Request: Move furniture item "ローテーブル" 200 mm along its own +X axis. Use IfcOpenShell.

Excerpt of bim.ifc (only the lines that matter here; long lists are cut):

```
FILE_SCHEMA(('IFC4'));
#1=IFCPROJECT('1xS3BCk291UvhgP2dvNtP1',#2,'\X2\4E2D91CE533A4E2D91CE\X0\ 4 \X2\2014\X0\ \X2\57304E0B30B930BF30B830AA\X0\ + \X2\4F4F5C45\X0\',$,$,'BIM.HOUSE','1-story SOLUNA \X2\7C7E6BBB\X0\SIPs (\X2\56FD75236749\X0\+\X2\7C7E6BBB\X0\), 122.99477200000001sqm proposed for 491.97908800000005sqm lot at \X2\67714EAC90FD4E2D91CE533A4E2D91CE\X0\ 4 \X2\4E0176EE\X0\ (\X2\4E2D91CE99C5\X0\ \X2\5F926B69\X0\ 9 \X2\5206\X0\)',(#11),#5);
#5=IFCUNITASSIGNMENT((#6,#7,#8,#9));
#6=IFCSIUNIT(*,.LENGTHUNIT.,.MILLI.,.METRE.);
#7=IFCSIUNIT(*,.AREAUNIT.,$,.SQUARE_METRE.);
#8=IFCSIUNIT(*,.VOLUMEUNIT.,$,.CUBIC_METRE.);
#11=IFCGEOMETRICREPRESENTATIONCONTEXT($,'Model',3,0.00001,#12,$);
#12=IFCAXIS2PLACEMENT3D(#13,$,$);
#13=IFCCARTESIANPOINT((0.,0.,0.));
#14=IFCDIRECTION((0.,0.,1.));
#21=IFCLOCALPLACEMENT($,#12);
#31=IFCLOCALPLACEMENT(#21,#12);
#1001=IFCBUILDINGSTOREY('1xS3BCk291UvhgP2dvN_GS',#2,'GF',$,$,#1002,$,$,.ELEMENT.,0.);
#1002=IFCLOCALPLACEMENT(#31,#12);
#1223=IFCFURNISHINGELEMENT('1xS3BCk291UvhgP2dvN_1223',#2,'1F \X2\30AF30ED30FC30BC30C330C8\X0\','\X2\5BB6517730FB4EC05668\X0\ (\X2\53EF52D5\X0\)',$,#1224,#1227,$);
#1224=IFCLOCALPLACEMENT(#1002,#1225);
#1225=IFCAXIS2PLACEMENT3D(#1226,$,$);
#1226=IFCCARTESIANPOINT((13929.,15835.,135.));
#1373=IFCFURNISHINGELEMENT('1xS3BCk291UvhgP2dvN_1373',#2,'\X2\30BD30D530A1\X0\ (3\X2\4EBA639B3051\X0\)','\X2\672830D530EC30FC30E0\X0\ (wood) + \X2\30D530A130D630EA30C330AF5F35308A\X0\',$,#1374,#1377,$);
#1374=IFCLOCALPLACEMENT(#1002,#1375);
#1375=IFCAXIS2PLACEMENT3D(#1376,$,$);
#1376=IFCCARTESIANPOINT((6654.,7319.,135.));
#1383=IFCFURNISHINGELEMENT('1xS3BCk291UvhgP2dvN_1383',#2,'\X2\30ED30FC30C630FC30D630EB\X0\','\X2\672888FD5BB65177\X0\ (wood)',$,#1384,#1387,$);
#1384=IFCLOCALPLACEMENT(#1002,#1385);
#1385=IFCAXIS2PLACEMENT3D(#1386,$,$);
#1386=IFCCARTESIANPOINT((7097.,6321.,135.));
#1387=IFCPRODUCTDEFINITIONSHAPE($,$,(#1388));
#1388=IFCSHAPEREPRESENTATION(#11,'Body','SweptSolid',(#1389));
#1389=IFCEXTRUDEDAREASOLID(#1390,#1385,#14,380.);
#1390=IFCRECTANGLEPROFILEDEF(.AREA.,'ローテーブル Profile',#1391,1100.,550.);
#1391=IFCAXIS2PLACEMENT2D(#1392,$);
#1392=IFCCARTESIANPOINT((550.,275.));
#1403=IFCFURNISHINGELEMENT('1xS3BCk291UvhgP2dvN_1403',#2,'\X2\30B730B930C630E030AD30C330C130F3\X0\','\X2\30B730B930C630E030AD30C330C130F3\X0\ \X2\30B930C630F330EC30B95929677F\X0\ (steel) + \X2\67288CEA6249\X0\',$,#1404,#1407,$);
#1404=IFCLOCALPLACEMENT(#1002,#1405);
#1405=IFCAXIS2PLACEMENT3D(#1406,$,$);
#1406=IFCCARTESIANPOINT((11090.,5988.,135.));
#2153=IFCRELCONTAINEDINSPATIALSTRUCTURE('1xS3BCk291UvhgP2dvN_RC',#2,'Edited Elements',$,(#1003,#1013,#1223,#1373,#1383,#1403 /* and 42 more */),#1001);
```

```python
import ifcopenshell
import ifcopenshell.api.geometry
import ifcopenshell.util.placement
import ifcopenshell.util.unit

model = ifcopenshell.open("bim.ifc")
unit_scale = ifcopenshell.util.unit.calculate_unit_scale(model)

item = model.by_id(1383)
matrix = ifcopenshell.util.placement.get_local_placement(item.ObjectPlacement)
matrix[:3, 3] += matrix[:3, 0] * 0.2 / unit_scale
ifcopenshell.api.geometry.edit_object_placement(model, product=item, matrix=matrix, is_si=False)

print(ifcopenshell.util.placement.get_local_placement(item.ObjectPlacement).round(3) + 0.0)

model.write("bim-out.ifc")
```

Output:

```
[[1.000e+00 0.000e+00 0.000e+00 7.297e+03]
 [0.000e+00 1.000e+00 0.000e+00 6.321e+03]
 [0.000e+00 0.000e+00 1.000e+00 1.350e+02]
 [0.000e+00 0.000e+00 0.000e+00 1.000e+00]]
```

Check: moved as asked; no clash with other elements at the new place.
